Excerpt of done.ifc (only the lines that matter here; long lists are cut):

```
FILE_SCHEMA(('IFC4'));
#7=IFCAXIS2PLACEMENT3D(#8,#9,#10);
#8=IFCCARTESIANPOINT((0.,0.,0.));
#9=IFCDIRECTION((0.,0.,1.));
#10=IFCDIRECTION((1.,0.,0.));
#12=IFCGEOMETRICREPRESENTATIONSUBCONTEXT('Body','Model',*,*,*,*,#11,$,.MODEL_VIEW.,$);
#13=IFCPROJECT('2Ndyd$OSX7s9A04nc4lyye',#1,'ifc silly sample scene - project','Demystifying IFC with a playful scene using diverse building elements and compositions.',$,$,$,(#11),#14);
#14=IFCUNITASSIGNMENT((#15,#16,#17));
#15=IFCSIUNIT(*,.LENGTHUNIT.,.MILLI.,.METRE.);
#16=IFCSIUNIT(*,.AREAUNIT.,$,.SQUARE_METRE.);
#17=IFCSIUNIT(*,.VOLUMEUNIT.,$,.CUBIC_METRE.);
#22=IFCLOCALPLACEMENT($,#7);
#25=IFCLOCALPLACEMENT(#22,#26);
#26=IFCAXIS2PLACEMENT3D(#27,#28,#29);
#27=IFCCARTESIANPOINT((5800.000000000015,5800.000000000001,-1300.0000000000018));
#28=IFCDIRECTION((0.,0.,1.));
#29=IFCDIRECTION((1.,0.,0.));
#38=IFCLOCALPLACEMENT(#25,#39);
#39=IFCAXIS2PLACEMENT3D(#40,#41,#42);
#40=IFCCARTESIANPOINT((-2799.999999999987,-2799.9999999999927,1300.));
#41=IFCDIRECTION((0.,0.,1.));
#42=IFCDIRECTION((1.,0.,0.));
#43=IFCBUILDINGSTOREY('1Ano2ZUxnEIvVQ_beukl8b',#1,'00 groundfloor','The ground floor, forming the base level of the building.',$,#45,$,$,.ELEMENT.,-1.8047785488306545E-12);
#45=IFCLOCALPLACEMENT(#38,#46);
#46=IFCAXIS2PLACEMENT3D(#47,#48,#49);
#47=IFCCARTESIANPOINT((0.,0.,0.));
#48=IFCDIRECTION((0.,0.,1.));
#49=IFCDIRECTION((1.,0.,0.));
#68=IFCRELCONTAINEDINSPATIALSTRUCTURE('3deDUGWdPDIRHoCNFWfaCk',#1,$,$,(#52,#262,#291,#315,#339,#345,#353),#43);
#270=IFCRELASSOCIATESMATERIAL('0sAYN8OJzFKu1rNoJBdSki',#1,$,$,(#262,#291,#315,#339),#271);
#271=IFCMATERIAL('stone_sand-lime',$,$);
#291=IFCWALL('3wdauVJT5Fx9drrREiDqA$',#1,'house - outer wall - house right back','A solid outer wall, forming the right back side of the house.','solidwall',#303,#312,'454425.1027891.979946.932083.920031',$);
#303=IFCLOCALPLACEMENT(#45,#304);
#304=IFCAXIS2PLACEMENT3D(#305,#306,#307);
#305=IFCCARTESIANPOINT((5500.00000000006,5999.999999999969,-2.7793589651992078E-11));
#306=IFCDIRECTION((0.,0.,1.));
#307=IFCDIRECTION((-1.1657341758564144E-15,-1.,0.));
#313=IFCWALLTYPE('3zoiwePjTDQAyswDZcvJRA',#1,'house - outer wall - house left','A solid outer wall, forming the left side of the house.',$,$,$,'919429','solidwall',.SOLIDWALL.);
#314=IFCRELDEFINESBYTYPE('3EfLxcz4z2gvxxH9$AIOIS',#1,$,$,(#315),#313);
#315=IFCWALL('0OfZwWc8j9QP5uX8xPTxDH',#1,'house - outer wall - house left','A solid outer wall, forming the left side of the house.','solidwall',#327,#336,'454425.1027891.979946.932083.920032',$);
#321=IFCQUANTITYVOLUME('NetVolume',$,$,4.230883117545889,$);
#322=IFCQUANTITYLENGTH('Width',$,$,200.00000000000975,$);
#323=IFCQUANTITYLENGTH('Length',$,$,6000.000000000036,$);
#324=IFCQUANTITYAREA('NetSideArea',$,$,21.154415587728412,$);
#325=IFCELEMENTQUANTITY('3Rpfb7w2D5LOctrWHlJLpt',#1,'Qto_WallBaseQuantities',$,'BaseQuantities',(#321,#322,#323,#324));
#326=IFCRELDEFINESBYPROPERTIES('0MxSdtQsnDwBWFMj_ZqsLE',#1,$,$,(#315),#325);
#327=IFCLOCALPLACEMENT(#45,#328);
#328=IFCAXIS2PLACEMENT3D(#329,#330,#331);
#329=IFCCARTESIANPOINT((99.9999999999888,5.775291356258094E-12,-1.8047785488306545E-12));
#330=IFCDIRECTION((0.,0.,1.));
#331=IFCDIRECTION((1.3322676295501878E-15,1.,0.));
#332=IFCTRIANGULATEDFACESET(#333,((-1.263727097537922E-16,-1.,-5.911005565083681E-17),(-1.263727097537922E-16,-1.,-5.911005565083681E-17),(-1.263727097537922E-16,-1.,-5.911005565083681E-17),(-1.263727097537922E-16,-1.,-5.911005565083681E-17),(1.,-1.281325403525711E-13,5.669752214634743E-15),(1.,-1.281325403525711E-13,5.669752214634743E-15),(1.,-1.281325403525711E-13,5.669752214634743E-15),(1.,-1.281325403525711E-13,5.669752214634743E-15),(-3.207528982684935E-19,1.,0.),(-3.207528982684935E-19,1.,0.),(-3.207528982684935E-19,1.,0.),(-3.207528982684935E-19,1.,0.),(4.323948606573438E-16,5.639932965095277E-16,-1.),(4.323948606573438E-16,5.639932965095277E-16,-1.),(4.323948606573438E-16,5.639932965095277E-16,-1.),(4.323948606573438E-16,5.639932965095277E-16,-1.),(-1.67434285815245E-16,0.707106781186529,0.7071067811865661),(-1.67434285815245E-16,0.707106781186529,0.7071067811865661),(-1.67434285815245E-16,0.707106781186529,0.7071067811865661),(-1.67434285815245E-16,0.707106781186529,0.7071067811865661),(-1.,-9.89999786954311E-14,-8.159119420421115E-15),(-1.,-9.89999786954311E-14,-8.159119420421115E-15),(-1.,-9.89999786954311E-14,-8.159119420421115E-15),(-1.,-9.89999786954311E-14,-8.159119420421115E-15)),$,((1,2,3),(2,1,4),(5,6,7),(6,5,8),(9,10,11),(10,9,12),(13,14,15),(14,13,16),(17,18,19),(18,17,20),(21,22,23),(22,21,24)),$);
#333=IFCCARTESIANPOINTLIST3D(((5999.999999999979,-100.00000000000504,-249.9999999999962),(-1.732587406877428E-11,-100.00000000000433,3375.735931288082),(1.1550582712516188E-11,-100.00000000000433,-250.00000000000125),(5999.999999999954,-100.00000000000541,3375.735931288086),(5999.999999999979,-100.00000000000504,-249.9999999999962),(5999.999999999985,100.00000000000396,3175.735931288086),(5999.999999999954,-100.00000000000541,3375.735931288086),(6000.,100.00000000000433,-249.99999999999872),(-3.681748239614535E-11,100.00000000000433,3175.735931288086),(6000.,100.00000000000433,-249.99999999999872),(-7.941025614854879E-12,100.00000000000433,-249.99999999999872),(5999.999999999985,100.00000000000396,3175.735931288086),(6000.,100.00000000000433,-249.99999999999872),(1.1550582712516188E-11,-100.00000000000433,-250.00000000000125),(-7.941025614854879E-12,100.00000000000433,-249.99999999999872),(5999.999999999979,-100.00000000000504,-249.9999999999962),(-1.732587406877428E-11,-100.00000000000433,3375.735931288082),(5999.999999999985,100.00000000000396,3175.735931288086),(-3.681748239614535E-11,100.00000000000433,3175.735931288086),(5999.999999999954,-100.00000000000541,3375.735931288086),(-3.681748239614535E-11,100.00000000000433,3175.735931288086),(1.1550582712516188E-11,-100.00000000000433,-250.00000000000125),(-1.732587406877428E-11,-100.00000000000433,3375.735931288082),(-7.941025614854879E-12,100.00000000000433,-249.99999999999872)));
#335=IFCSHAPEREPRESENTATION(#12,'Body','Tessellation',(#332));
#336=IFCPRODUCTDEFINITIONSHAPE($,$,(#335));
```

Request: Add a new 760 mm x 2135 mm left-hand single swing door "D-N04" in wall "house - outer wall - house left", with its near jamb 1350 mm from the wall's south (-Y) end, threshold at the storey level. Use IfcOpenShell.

```python
import numpy as np
import ifcopenshell
import ifcopenshell.api.feature
import ifcopenshell.api.geometry
import ifcopenshell.api.pset
import ifcopenshell.api.root
import ifcopenshell.api.spatial
import ifcopenshell.geom
import ifcopenshell.util.element
import ifcopenshell.util.placement
import ifcopenshell.util.representation
import ifcopenshell.util.shape
import ifcopenshell.util.unit

model = ifcopenshell.open("done.ifc")
unit_scale = ifcopenshell.util.unit.calculate_unit_scale(model)
area_scale = ifcopenshell.util.unit.calculate_unit_scale(model, "AREAUNIT")
volume_scale = ifcopenshell.util.unit.calculate_unit_scale(model, "VOLUMEUNIT")
settings = ifcopenshell.geom.settings()


def volume(element):
    """Net volume in cubic metres, openings subtracted."""
    shape = ifcopenshell.geom.create_shape(settings, element)
    return ifcopenshell.util.shape.get_volume(shape.geometry)


wall = model.by_guid("0OfZwWc8j9QP5uX8xPTxDH")
storey = ifcopenshell.util.element.get_container(wall, ifc_class="IfcBuildingStorey")
context = ifcopenshell.util.representation.get_context(model, "Model", "Body", "MODEL_VIEW")
before = volume(wall)

width, height, from_end, sill = 0.76, 2.135, 1.35, 0.0  # metres

# The wall runs along its own X axis, and the end named is its -X end.
wall_shape = ifcopenshell.geom.create_shape(settings, wall)
x, y, z = ifcopenshell.util.shape.get_vertices(wall_shape.geometry).T
start = x.min() + from_end
face, thickness = float(y.min()), float(y.max() - y.min())
wall_matrix = ifcopenshell.util.placement.get_local_placement(wall.ObjectPlacement)
level = ifcopenshell.util.placement.get_local_placement(storey.ObjectPlacement)[2, 3]


def in_wall(x, y):
    """Placement at x, y metres in the wall's axes, at sill height."""
    matrix = wall_matrix.copy()
    matrix[:, 3] = wall_matrix @ np.array([x / unit_scale, y / unit_scale, 0.0, 1.0])
    matrix[2, 3] = level + sill / unit_scale
    return matrix


# Opening: a box that overshoots both wall faces by 50 mm.
opening = ifcopenshell.api.root.create_entity(model, ifc_class="IfcOpeningElement", predefined_type="OPENING")
box = ifcopenshell.api.geometry.add_wall_representation(
    model, context=context, length=width, height=height, thickness=thickness + 0.1
)
ifcopenshell.api.geometry.assign_representation(model, product=opening, representation=box)
ifcopenshell.api.geometry.edit_object_placement(model, product=opening, matrix=in_wall(start, face - 0.05), is_si=False)
ifcopenshell.api.feature.add_feature(model, feature=opening, element=wall)

door = ifcopenshell.api.root.create_entity(model, ifc_class="IfcDoor", name="D-N04", predefined_type="DOOR")
door.OverallWidth, door.OverallHeight = width / unit_scale, height / unit_scale
door.OperationType = "SINGLE_SWING_LEFT"
body = ifcopenshell.api.geometry.add_door_representation(
    model,
    context=context,
    overall_width=door.OverallWidth,
    overall_height=door.OverallHeight,
    operation_type="SINGLE_SWING_LEFT",
    lining_properties={"LiningDepth": thickness / unit_scale, "ThresholdDepth": thickness / unit_scale},
)
ifcopenshell.api.geometry.assign_representation(model, product=door, representation=body)
ifcopenshell.api.spatial.assign_container(model, products=[door], relating_structure=storey)
ifcopenshell.api.feature.add_filling(model, opening=opening, element=door)

# The lining spans the wall, so the door starts at the wall face.
ifcopenshell.api.geometry.edit_object_placement(model, product=door, matrix=in_wall(start, face), is_si=False)

after = volume(wall)

# Update the wall's stored quantities.
qto = model.by_id(ifcopenshell.util.element.get_pset(wall, "Qto_WallBaseQuantities", should_inherit=False)["id"])
ifcopenshell.api.pset.edit_qto(model, qto=qto, properties={
    "NetVolume": after / volume_scale,
    "NetSideArea": after / thickness / area_scale,
})

print(f"wall volume {before:.3f} -> {after:.3f} m3")

model.write("done_updated.ifc")
```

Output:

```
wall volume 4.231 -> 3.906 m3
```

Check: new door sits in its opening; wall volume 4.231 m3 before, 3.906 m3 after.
